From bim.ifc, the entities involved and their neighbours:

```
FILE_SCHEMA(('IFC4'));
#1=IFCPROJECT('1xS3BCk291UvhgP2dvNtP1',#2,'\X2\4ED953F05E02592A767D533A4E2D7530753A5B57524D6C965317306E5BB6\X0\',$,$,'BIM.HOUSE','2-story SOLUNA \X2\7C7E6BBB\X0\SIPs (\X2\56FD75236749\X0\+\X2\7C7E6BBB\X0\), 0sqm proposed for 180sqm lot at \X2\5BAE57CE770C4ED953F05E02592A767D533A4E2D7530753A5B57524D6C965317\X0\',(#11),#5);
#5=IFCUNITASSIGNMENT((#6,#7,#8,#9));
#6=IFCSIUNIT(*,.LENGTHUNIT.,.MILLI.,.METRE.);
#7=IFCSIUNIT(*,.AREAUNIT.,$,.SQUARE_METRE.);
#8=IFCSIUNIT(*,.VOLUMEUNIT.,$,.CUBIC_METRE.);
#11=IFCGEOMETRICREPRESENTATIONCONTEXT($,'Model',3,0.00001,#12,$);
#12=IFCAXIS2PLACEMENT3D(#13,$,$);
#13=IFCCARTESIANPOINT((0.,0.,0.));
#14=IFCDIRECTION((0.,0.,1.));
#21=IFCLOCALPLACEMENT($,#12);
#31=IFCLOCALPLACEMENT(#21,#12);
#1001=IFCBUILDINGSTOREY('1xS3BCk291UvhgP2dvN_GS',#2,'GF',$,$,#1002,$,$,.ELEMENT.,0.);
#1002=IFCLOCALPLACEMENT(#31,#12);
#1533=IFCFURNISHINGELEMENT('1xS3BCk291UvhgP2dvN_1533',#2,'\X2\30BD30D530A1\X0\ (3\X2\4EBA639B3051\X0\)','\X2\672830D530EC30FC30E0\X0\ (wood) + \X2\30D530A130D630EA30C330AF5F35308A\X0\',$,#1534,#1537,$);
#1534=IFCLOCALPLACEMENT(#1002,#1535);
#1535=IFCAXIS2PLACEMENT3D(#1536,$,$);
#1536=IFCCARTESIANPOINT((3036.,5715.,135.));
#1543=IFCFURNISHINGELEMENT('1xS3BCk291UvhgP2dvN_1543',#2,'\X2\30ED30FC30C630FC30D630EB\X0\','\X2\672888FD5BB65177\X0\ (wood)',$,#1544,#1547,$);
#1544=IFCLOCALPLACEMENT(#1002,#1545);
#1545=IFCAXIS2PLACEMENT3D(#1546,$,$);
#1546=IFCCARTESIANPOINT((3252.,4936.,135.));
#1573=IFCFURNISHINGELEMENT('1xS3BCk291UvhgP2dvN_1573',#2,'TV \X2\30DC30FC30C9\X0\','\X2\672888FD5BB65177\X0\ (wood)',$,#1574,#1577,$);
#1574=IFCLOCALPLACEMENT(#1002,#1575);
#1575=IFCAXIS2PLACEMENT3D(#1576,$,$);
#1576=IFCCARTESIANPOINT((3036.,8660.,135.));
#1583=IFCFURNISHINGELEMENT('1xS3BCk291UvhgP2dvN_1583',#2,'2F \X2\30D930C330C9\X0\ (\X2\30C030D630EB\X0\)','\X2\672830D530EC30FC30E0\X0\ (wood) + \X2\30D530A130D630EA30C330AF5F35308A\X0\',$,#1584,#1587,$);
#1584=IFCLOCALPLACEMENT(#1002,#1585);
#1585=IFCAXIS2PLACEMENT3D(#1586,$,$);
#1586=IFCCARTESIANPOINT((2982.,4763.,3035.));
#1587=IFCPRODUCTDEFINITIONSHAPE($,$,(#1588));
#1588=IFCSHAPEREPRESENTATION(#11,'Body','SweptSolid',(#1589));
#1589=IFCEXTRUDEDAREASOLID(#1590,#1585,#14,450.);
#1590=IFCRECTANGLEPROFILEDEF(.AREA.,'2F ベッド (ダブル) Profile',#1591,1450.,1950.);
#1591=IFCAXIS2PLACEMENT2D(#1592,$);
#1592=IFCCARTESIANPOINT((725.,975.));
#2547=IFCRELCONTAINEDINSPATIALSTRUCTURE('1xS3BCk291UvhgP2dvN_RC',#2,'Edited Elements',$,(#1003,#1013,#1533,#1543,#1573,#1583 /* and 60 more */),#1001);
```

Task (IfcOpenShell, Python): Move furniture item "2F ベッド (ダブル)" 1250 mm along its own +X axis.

```python
import ifcopenshell
import ifcopenshell.api.geometry
import ifcopenshell.util.placement
import ifcopenshell.util.unit

model = ifcopenshell.open("bim.ifc")
unit_scale = ifcopenshell.util.unit.calculate_unit_scale(model)

item = model.by_guid("1xS3BCk291UvhgP2dvN_1583")
matrix = ifcopenshell.util.placement.get_local_placement(item.ObjectPlacement)
matrix[:3, 3] += matrix[:3, 0] * 1.25 / unit_scale
ifcopenshell.api.geometry.edit_object_placement(model, product=item, matrix=matrix, is_si=False)

print(ifcopenshell.util.placement.get_local_placement(item.ObjectPlacement).round(3) + 0.0)

model.write("bim_rev.ifc")
```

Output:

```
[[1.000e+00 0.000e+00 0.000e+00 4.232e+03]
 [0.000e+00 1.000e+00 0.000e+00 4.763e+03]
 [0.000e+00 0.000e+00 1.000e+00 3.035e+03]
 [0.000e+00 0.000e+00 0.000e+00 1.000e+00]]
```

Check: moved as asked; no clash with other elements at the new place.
